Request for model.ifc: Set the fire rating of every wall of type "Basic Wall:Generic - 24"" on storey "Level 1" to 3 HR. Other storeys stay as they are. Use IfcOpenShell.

First a look at what the model holds.

```python
import ifcopenshell
import ifcopenshell.util.element

model = ifcopenshell.open("model.ifc")
print(model.schema)
storey = next(s for s in model.by_type("IfcBuildingStorey") if s.Name == "Level 1")
walls = [e for e in ifcopenshell.util.element.get_decomposition(storey) if e.is_a("IfcWall")]
seen = {}
for e in walls:
    element_type = ifcopenshell.util.element.get_type(e)
    key = (element_type.Name if element_type != e and element_type else None, ifcopenshell.util.element.get_pset(e, "Pset_WallCommon", "FireRating"))
    seen[key] = seen.get(key, 0) + 1
for (name, value), count in sorted(seen.items(), key=str):
    print(count, "x", name, "|", value)
```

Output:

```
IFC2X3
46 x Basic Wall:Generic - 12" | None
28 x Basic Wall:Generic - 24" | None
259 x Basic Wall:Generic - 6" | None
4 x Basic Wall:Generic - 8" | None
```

```python
import ifcopenshell
import ifcopenshell.api.pset
import ifcopenshell.util.element

model = ifcopenshell.open("model.ifc")

storey = next(s for s in model.by_type("IfcBuildingStorey") if s.Name == "Level 1")
walls = [e for e in ifcopenshell.util.element.get_decomposition(storey) if e.is_a("IfcWall")]

count = 0
for e in walls:
    element_type = ifcopenshell.util.element.get_type(e)
    if element_type in (None, e) or element_type.Name != 'Basic Wall:Generic - 24"':
        continue
    # add_pset returns the element's existing set when there is one.
    pset = ifcopenshell.api.pset.add_pset(model, product=e, name="Pset_WallCommon")
    ifcopenshell.api.pset.edit_pset(model, pset=pset, properties={"FireRating": "3 HR"})
    count += 1

print(count, "walls updated")

model.write("model_rev.ifc")
```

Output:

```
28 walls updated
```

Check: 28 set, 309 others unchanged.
